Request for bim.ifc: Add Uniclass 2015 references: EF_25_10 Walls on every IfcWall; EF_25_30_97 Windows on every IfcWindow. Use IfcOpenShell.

First a look at what the model holds.

```python
import ifcopenshell

model = ifcopenshell.open("bim.ifc")
print(model.schema)
print("classifications:", [c.Name for c in model.by_type("IfcClassification")])
for ifc_class in ("IfcDoor", "IfcRoof", "IfcStair", "IfcWall", "IfcWindow"):
    print(ifc_class, len(model.by_type(ifc_class)))
```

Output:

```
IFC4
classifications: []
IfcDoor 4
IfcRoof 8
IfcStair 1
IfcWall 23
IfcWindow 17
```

```python
import ifcopenshell
import ifcopenshell.api.classification

model = ifcopenshell.open("bim.ifc")

system = ifcopenshell.api.classification.add_classification(model, classification="Uniclass 2015")

codes = {
    "IfcWall": ("EF_25_10", "Walls"),
    "IfcWindow": ("EF_25_30_97", "Windows"),
}
for ifc_class, (code, name) in codes.items():
    products = model.by_type(ifc_class)
    ifcopenshell.api.classification.add_reference(
        model, products=products, classification=system, identification=code, name=name
    )
    print(code, len(products))

model.write("bim_updated.ifc")
```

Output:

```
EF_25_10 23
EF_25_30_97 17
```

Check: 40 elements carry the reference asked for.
